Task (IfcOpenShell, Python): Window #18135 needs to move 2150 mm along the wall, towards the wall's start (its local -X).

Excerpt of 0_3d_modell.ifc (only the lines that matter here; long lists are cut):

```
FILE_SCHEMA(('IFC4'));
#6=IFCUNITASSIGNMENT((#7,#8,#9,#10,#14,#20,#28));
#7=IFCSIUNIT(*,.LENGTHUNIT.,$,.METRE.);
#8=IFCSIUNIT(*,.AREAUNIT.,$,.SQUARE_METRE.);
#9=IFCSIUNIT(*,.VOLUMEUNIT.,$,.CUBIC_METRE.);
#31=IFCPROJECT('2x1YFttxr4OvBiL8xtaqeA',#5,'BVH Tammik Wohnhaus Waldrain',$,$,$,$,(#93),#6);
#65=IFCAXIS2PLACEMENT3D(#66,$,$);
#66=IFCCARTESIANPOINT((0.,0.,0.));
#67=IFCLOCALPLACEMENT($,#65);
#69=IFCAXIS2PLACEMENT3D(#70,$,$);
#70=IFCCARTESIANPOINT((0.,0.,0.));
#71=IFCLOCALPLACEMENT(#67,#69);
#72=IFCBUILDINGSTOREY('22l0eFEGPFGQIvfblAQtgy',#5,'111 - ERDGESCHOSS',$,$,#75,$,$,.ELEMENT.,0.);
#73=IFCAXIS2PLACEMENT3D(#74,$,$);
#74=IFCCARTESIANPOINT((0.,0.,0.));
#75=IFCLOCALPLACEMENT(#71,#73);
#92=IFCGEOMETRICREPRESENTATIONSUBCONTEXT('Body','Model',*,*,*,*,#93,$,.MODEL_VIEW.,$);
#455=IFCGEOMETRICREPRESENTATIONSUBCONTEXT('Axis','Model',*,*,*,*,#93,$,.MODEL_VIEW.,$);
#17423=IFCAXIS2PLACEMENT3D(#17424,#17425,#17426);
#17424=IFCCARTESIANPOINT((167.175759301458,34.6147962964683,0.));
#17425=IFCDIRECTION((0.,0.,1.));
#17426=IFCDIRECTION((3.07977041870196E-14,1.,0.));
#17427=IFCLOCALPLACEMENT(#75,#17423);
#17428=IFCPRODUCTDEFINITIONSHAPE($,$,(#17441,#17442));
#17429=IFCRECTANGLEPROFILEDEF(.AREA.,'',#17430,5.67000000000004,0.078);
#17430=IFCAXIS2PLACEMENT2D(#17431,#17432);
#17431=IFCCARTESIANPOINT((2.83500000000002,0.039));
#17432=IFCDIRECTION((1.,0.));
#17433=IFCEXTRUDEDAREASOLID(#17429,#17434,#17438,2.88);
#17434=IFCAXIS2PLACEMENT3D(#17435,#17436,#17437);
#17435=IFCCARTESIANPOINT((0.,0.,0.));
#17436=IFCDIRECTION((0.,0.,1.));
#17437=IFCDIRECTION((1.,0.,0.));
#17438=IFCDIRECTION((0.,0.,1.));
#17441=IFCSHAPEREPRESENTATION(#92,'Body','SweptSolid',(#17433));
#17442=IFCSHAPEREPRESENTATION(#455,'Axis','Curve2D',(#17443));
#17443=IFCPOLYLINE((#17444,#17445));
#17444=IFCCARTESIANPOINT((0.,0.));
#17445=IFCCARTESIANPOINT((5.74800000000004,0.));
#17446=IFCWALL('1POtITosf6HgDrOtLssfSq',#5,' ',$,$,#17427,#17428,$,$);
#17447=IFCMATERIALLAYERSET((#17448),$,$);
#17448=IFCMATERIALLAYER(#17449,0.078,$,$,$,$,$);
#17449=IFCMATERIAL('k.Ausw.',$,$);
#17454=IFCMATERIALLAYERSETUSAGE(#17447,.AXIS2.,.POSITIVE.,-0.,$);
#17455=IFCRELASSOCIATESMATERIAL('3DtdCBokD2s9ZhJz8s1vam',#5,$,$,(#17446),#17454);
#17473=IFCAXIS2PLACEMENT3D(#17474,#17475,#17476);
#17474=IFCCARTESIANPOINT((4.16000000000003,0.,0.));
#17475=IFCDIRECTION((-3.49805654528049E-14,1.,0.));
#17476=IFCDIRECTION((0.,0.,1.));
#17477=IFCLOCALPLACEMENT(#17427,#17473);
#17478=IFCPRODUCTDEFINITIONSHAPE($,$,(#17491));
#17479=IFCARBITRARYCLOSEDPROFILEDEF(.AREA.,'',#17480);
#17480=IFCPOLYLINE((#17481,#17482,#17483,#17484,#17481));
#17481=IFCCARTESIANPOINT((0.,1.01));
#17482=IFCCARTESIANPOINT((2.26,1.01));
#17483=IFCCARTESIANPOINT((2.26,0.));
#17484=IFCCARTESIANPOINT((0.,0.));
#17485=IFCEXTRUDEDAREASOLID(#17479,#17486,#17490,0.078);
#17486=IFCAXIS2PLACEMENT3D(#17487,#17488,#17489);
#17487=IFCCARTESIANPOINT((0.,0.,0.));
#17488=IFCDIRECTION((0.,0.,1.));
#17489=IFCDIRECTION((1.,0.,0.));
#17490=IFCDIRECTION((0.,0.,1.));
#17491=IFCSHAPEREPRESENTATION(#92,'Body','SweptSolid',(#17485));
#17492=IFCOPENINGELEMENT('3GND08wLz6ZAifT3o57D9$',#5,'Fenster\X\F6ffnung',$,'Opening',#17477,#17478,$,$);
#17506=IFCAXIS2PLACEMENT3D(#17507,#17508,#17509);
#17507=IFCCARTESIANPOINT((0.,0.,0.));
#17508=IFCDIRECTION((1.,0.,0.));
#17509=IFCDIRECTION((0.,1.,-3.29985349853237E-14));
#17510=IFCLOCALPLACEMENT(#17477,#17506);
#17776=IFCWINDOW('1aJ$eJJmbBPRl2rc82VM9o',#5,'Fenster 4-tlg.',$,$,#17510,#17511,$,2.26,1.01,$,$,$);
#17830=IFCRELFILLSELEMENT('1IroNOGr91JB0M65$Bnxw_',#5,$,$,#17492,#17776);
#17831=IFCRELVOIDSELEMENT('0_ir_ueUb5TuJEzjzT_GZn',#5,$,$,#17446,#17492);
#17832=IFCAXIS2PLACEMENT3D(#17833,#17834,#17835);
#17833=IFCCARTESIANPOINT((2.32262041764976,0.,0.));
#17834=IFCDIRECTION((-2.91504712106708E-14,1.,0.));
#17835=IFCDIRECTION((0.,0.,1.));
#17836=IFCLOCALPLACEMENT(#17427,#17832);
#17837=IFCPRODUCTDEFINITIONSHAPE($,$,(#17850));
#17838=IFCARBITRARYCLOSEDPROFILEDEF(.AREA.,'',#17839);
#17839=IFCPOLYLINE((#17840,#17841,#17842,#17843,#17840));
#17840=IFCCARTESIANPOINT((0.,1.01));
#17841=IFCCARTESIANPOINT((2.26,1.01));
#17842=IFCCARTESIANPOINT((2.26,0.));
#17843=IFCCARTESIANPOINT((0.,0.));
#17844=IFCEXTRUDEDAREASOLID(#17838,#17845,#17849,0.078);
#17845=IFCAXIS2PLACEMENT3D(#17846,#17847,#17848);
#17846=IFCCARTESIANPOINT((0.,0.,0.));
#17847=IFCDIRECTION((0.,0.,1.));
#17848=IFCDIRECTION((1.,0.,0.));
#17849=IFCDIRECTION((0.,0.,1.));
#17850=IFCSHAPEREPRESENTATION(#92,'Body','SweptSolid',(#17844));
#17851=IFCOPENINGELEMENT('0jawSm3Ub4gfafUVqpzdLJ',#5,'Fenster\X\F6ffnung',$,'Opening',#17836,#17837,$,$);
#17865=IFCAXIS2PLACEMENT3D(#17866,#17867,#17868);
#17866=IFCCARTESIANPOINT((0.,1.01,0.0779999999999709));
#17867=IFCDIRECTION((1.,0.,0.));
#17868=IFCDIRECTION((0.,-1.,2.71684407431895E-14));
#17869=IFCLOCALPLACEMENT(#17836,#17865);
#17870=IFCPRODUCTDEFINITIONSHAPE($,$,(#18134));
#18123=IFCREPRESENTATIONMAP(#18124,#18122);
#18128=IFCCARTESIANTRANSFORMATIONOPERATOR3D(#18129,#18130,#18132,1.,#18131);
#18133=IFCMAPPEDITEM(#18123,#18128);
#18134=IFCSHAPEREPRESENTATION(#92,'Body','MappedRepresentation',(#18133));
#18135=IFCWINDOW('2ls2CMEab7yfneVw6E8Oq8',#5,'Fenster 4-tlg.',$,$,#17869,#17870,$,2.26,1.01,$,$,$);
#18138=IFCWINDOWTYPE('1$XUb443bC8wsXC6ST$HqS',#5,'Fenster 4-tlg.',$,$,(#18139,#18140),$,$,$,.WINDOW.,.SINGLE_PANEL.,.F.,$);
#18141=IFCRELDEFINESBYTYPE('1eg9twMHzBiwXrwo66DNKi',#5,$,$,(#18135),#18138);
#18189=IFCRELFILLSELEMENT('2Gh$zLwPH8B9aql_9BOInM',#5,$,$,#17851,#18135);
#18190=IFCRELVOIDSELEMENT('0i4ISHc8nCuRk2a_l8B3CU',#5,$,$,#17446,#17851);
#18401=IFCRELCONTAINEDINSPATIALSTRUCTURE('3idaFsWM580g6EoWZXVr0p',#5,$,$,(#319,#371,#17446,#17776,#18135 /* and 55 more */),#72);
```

```python
import ifcopenshell
import ifcopenshell.api.geometry
import ifcopenshell.util.placement

model = ifcopenshell.open("0_3d_modell.ifc")

window = model.by_guid("2ls2CMEab7yfneVw6E8Oq8")
opening = window.FillsVoids[0].RelatingOpeningElement
wall = opening.VoidsElements[0].RelatingBuildingElement

wall_matrix = ifcopenshell.util.placement.get_local_placement(wall.ObjectPlacement)
shift = wall_matrix[:3, 0] * -2.15
before = ifcopenshell.util.placement.get_local_placement(window.ObjectPlacement)[:3, 3].copy()

# The window is placed relative to its opening, so it follows when the opening moves.
matrix = ifcopenshell.util.placement.get_local_placement(opening.ObjectPlacement)
matrix[:3, 3] += shift
ifcopenshell.api.geometry.edit_object_placement(
    model, product=opening, matrix=matrix, is_si=False, should_transform_children=True
)

after = ifcopenshell.util.placement.get_local_placement(window.ObjectPlacement)[:3, 3]
print("window moved by", (after - before).round(3) + 0.0)

model.write("0_3d_modell_updated.ifc")
```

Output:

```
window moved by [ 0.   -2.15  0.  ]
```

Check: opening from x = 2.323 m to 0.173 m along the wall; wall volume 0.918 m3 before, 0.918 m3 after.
